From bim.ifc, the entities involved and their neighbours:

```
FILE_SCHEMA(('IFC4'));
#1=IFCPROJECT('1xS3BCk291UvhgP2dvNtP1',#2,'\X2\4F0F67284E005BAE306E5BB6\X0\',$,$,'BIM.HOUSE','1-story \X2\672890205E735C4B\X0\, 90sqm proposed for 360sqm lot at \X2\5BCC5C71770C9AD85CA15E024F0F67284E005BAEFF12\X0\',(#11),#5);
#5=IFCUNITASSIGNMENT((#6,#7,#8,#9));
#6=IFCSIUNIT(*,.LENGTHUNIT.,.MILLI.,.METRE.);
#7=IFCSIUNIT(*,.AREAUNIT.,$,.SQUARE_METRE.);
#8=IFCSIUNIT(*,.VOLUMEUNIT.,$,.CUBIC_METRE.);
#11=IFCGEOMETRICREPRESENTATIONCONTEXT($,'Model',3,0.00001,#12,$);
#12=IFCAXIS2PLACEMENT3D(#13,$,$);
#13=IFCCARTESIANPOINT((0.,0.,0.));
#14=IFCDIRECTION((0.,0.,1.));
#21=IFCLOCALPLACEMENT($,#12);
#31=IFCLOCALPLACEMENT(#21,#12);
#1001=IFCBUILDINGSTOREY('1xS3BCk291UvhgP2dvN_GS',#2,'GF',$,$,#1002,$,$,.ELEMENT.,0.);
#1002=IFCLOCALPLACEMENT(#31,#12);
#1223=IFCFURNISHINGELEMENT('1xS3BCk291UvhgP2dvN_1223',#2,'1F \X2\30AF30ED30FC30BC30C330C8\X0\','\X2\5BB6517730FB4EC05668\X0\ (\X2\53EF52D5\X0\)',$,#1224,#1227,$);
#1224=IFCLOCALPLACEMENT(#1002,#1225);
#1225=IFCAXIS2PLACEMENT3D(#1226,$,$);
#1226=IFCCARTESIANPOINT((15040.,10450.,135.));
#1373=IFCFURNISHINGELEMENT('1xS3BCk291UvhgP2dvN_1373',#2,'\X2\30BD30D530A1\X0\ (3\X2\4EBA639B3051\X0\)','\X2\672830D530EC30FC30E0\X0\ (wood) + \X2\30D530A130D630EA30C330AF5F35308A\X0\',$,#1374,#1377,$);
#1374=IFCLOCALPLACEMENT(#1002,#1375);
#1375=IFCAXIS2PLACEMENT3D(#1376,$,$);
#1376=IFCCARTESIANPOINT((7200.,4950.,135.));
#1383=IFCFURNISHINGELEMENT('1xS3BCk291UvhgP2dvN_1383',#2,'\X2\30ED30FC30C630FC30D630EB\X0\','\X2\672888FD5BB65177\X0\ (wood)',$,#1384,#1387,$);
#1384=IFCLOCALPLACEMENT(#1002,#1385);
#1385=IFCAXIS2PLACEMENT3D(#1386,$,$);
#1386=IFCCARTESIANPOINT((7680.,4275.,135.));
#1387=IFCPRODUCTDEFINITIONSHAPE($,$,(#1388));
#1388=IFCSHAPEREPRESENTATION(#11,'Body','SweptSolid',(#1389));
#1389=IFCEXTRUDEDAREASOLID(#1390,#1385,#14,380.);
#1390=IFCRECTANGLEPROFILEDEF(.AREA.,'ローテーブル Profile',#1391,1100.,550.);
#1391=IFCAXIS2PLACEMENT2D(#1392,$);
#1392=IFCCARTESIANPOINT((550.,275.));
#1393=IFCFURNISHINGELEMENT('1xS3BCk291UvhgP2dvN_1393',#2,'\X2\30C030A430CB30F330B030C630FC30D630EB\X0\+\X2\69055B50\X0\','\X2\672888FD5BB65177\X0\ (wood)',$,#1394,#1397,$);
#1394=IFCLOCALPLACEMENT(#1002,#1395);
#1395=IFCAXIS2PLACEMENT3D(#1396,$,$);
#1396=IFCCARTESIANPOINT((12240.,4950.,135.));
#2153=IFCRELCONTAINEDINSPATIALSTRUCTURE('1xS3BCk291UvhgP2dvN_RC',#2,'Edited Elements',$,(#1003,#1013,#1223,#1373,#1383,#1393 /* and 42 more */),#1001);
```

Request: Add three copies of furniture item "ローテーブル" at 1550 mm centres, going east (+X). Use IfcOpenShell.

```python
import numpy as np
import ifcopenshell
import ifcopenshell.api.geometry
import ifcopenshell.api.root
import ifcopenshell.util.element
import ifcopenshell.util.placement
import ifcopenshell.util.unit

model = ifcopenshell.open("bim.ifc")
unit_scale = ifcopenshell.util.unit.calculate_unit_scale(model)


def reuse_history(source, copy):
    """copy_class also copies each property set's owner history, people and application; keep the originals."""
    for rel in copy.IsDefinedBy:
        if rel.is_a("IfcRelDefinesByProperties") and (history := rel.RelatingPropertyDefinition.OwnerHistory):
            rel.RelatingPropertyDefinition.OwnerHistory = source.OwnerHistory
            ifcopenshell.util.element.remove_deep2(model, history)


source = model.by_id(1383)
base = ifcopenshell.util.placement.get_local_placement(source.ObjectPlacement)
step = np.array([1.0, 0.0, 0.0]) * 1.55 / unit_scale

for i in range(1, 4):
    copy = ifcopenshell.api.root.copy_class(model, product=source)
    copy.Representation = ifcopenshell.util.element.copy_deep(
        model, source.Representation, exclude=["IfcGeometricRepresentationContext", "IfcRepresentationMap"]
    )
    reuse_history(source, copy)
    matrix = base.copy()
    matrix[:3, 3] += i * step
    print("added at", matrix[:3, 3].round(3) + 0.0)
    ifcopenshell.api.geometry.edit_object_placement(model, product=copy, matrix=matrix, is_si=False)

model.write("bim_v2.ifc")
```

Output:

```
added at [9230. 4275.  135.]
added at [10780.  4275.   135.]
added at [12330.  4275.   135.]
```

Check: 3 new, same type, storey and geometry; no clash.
